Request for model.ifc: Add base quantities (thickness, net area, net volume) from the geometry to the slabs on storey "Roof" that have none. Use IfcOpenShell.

First a look at what the model holds.

```python
import ifcopenshell
import ifcopenshell.util.element
import ifcopenshell.util.unit

model = ifcopenshell.open("model.ifc")
print(model.schema)
for unit_type in ("LENGTHUNIT", "AREAUNIT", "VOLUMEUNIT"):
    print(unit_type, ifcopenshell.util.unit.calculate_unit_scale(model, unit_type))
storey = next(s for s in model.by_type("IfcBuildingStorey") if s.Name == "Roof")
slabs = [e for e in ifcopenshell.util.element.get_decomposition(storey) if e.is_a("IfcSlab")]
for e in sorted(slabs, key=lambda e: e.id()):
    print(e.id(), e.is_a(), e.Name, list(ifcopenshell.util.element.get_psets(e, qtos_only=True)), sep=" | ")
```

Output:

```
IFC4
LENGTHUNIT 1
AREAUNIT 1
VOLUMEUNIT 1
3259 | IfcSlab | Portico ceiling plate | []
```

```python
import ifcopenshell
import ifcopenshell.api.pset
import ifcopenshell.geom
import ifcopenshell.util.element
import ifcopenshell.util.shape
import ifcopenshell.util.unit

model = ifcopenshell.open("model.ifc")
unit_scale = ifcopenshell.util.unit.calculate_unit_scale(model)
area_scale = ifcopenshell.util.unit.calculate_unit_scale(model, "AREAUNIT")
volume_scale = ifcopenshell.util.unit.calculate_unit_scale(model, "VOLUMEUNIT")
settings = ifcopenshell.geom.settings()

storey = next(s for s in model.by_type("IfcBuildingStorey") if s.Name == "Roof")
slabs = [e for e in ifcopenshell.util.element.get_decomposition(storey) if e.is_a("IfcSlab")]

for e in sorted(slabs, key=lambda e: e.id()):
    if ifcopenshell.util.element.get_psets(e, qtos_only=True, should_inherit=False):
        continue
    # Geometry comes back in metres, in the element's own axes.
    shape = ifcopenshell.geom.create_shape(settings, e)
    values = {
        "Width": ifcopenshell.util.shape.get_z(shape.geometry) / unit_scale,
        "NetArea": ifcopenshell.util.shape.get_footprint_area(shape.geometry) / area_scale,
        "NetVolume": ifcopenshell.util.shape.get_volume(shape.geometry) / volume_scale,
    }
    qto = ifcopenshell.api.pset.add_qto(model, product=e, name="Qto_SlabBaseQuantities")
    ifcopenshell.api.pset.edit_qto(model, qto=qto, properties=values)
    print(e.id(), {k: round(v, 3) for k, v in values.items()})

model.write("model_edited.ifc")
```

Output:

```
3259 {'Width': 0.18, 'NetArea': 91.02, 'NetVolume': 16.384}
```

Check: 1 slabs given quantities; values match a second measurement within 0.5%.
